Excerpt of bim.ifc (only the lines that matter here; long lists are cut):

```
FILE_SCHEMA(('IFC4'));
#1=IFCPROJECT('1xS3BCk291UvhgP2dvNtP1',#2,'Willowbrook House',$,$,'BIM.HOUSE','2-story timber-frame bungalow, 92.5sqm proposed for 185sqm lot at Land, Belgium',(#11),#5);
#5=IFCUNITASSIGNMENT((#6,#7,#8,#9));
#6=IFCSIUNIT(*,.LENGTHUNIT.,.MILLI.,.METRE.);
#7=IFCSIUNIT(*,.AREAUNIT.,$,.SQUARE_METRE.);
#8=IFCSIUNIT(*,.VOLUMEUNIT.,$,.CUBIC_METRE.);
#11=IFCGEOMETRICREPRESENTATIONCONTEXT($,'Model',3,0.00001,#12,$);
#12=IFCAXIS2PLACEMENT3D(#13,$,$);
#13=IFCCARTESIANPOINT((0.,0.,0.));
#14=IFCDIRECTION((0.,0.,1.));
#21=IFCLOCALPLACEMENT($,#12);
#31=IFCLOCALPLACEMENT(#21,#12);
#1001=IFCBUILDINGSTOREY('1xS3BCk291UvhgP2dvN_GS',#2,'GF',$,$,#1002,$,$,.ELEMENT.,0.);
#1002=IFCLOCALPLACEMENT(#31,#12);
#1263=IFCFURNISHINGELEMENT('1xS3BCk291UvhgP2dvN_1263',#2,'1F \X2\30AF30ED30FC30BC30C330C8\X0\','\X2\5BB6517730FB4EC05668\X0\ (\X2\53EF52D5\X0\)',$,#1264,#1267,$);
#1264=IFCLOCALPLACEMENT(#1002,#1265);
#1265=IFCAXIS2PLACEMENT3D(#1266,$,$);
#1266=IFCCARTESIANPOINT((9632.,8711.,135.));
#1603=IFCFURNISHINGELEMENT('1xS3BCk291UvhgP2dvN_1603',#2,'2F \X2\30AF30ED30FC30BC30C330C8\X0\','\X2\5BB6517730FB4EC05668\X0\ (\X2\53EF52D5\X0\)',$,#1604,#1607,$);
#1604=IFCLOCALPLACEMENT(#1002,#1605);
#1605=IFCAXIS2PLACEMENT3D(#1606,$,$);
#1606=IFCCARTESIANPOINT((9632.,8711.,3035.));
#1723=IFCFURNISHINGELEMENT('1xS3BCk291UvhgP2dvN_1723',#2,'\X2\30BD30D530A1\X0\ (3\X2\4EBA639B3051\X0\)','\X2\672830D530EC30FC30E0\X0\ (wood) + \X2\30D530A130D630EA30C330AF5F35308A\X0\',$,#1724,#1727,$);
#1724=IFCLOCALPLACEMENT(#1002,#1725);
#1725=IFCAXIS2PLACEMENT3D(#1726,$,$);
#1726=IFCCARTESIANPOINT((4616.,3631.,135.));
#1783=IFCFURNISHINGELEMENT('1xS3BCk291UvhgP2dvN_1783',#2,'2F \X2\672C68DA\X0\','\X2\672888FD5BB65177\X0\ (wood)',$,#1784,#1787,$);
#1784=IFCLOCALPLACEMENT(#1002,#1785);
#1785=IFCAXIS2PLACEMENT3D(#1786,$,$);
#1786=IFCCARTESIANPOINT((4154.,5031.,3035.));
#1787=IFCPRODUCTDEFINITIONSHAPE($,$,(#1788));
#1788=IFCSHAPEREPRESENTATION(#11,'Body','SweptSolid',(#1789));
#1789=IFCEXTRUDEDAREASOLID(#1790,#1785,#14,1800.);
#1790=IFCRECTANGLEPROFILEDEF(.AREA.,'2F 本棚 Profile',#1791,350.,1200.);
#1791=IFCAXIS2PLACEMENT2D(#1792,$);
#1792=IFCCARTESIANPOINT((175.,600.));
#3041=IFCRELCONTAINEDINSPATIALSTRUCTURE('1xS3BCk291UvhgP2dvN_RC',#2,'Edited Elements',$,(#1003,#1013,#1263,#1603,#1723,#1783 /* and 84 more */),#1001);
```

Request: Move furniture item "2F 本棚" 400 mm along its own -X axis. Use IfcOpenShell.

```python
import ifcopenshell
import ifcopenshell.api.geometry
import ifcopenshell.util.placement

model = ifcopenshell.open("bim.ifc")

item = model.by_guid("1xS3BCk291UvhgP2dvN_1783")
matrix = ifcopenshell.util.placement.get_local_placement(item.ObjectPlacement)
matrix[:3, 3] -= matrix[:3, 0] * 400.0
ifcopenshell.api.geometry.edit_object_placement(model, product=item, matrix=matrix, is_si=False)

print(ifcopenshell.util.placement.get_local_placement(item.ObjectPlacement).round(3) + 0.0)

model.write("bim_v2.ifc")
```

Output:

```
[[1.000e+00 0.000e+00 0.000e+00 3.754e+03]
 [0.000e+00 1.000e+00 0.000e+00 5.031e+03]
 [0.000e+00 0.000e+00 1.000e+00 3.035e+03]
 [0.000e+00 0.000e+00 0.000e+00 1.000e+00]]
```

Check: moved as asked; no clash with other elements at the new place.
